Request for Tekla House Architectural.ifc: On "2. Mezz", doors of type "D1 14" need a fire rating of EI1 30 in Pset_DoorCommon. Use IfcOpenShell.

First a look at what the model holds.

```python
import ifcopenshell
import ifcopenshell.util.element

model = ifcopenshell.open("Tekla House Architectural.ifc")
print(model.schema)
storey = next(s for s in model.by_type("IfcBuildingStorey") if s.Name == "2. Mezz")
doors = [e for e in ifcopenshell.util.element.get_decomposition(storey) if e.is_a("IfcDoor")]
seen = {}
for e in doors:
    element_type = ifcopenshell.util.element.get_type(e)
    key = (element_type.Name if element_type != e and element_type else None, ifcopenshell.util.element.get_pset(e, "Pset_DoorCommon", "FireRating"))
    seen[key] = seen.get(key, 0) + 1
for (name, value), count in sorted(seen.items(), key=str):
    print(count, "x", name, "|", value)
```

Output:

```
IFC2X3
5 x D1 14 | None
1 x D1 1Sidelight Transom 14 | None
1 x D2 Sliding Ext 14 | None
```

```python
import ifcopenshell
import ifcopenshell.api.pset
import ifcopenshell.util.element

model = ifcopenshell.open("Tekla House Architectural.ifc")

storey = next(s for s in model.by_type("IfcBuildingStorey") if s.Name == "2. Mezz")
doors = [e for e in ifcopenshell.util.element.get_decomposition(storey) if e.is_a("IfcDoor")]

count = 0
for e in doors:
    element_type = ifcopenshell.util.element.get_type(e)
    if element_type in (None, e) or element_type.Name != "D1 14":
        continue
    # add_pset returns the element's existing set when there is one.
    pset = ifcopenshell.api.pset.add_pset(model, product=e, name="Pset_DoorCommon")
    ifcopenshell.api.pset.edit_pset(model, pset=pset, properties={"FireRating": "EI1 30"})
    count += 1

print(count, "doors updated")

model.write("Tekla House Architectural-out.ifc")
```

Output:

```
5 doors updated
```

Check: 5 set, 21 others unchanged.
